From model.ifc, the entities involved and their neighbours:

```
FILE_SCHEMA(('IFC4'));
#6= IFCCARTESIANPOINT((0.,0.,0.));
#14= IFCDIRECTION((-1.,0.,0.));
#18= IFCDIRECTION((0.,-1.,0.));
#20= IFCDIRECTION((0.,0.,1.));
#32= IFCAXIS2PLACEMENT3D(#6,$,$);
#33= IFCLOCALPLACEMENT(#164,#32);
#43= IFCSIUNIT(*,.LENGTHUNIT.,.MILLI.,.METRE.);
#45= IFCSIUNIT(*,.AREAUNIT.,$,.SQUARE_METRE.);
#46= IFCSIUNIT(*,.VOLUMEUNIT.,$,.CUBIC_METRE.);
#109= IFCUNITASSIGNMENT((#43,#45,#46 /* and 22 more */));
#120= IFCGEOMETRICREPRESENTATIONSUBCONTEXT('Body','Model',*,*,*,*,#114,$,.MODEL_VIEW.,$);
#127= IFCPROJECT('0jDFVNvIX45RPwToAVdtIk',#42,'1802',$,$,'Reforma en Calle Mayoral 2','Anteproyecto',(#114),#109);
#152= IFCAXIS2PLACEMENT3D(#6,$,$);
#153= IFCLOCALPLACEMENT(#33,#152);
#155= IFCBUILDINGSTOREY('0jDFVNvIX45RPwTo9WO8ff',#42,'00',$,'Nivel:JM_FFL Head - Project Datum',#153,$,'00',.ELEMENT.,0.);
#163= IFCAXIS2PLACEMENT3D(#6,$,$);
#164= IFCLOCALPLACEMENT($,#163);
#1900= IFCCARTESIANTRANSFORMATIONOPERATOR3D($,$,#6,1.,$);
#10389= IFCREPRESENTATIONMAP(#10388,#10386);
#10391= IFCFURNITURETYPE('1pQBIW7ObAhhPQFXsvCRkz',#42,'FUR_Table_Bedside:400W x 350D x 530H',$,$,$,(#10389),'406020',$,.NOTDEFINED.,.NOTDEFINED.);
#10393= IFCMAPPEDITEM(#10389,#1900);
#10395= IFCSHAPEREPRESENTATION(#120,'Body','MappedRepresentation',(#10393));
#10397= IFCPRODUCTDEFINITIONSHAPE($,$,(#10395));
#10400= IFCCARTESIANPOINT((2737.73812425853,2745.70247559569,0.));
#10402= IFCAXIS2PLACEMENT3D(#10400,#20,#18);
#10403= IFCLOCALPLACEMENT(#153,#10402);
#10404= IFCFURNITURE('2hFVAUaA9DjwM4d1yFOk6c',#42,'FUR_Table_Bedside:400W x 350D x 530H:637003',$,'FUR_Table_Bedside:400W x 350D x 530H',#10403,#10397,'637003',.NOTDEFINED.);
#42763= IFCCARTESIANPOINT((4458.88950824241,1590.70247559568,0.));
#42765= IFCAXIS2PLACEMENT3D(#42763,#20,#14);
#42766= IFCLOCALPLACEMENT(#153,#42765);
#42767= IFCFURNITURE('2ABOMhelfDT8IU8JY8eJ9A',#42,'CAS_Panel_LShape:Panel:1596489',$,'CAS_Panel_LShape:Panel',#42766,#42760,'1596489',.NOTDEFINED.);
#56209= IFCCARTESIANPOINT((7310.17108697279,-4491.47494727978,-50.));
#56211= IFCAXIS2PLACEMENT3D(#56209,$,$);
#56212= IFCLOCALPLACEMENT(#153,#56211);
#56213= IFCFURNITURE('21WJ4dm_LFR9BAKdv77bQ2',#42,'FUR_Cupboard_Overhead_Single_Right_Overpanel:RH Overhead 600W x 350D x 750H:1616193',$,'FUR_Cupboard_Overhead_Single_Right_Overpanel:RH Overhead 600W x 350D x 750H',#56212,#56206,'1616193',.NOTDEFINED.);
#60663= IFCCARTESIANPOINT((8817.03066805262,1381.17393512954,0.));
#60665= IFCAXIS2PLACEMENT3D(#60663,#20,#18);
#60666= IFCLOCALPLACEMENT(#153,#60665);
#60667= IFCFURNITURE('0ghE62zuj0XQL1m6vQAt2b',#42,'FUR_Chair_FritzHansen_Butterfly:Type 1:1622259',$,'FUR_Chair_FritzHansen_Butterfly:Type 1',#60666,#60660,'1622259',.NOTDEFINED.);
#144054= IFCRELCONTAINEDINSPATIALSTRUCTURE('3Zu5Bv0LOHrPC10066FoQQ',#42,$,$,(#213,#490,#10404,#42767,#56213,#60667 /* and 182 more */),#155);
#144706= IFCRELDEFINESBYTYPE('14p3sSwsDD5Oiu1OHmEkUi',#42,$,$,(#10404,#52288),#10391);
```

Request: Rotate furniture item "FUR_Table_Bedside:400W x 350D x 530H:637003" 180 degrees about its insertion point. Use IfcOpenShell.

```python
import ifcopenshell
import ifcopenshell.api.geometry
import ifcopenshell.util.placement

model = ifcopenshell.open("model.ifc")

item = model.by_guid("2hFVAUaA9DjwM4d1yFOk6c")
matrix = ifcopenshell.util.placement.get_local_placement(item.ObjectPlacement)
matrix = matrix @ ifcopenshell.util.placement.rotation(180, "Z")
ifcopenshell.api.geometry.edit_object_placement(model, product=item, matrix=matrix, is_si=False)

print(ifcopenshell.util.placement.get_local_placement(item.ObjectPlacement).round(3) + 0.0)

model.write("model_v2.ifc")
```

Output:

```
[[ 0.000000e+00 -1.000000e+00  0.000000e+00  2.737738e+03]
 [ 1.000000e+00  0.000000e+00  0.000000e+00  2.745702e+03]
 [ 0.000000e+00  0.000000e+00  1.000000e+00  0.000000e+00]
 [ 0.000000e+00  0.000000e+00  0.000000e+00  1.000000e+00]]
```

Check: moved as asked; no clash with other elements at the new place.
